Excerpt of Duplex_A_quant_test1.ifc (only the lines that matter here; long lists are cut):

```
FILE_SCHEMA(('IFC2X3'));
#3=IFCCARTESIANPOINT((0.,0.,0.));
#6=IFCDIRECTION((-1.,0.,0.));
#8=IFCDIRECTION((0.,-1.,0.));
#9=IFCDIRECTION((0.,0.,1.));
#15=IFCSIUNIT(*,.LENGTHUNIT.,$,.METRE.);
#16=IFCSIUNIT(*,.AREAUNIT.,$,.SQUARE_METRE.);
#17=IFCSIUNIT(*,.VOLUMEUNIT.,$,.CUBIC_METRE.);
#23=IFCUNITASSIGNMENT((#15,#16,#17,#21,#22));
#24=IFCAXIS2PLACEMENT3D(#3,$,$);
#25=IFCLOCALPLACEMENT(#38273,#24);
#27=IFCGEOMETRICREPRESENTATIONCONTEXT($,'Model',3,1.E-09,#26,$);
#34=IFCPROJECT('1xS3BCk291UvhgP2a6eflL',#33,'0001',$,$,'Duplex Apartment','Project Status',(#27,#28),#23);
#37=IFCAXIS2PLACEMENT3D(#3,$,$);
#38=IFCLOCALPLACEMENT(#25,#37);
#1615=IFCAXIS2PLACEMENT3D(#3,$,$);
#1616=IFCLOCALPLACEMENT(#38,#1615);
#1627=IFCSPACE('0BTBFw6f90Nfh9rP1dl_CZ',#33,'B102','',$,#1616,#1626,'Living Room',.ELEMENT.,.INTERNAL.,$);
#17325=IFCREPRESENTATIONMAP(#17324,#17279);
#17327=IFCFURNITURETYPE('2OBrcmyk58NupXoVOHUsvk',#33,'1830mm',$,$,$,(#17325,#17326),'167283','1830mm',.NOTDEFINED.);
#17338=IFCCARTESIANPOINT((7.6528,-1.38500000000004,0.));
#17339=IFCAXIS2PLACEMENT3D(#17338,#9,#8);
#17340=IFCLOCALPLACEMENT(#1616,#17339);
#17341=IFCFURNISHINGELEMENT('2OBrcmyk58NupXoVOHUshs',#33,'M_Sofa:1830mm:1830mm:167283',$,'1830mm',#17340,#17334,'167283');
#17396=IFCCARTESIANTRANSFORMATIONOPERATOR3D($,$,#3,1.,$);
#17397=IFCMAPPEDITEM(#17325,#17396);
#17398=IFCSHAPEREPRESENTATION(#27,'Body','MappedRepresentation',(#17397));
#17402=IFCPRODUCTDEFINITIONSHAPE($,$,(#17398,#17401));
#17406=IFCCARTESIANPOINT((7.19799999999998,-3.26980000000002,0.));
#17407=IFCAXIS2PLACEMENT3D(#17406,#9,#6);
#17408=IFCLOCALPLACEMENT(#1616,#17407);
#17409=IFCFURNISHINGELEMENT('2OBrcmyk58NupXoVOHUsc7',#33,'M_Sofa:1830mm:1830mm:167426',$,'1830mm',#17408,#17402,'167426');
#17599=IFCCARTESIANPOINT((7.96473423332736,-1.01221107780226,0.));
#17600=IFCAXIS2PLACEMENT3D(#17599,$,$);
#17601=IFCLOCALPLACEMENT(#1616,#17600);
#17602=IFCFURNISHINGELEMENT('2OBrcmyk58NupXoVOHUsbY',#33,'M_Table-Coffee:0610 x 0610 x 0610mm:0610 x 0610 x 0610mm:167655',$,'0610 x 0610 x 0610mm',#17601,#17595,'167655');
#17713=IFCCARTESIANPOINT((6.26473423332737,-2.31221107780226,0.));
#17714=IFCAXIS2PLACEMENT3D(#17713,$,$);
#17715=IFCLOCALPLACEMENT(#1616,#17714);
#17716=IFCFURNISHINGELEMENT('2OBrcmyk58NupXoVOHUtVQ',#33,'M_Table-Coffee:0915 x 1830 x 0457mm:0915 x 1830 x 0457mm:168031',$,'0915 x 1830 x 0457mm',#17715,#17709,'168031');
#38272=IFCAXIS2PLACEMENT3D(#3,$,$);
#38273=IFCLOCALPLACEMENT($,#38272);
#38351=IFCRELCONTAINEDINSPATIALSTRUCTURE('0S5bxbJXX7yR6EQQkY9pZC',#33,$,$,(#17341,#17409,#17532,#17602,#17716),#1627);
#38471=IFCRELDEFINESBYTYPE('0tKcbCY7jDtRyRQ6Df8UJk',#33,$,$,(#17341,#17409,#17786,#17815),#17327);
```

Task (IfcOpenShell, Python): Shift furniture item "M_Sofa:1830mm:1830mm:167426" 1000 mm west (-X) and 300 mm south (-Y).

```python
import ifcopenshell
import ifcopenshell.api.geometry
import ifcopenshell.util.placement

model = ifcopenshell.open("Duplex_A_quant_test1.ifc")

item = model.by_guid("2OBrcmyk58NupXoVOHUsc7")
matrix = ifcopenshell.util.placement.get_local_placement(item.ObjectPlacement)
matrix[0, 3] -= 1.0
matrix[1, 3] -= 0.3
ifcopenshell.api.geometry.edit_object_placement(model, product=item, matrix=matrix, is_si=False)

print(ifcopenshell.util.placement.get_local_placement(item.ObjectPlacement).round(3) + 0.0)

model.write("Duplex_A_quant_test1_rev.ifc")
```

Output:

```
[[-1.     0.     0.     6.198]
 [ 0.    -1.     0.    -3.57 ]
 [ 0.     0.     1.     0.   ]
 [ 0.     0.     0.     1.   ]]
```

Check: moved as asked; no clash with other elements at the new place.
